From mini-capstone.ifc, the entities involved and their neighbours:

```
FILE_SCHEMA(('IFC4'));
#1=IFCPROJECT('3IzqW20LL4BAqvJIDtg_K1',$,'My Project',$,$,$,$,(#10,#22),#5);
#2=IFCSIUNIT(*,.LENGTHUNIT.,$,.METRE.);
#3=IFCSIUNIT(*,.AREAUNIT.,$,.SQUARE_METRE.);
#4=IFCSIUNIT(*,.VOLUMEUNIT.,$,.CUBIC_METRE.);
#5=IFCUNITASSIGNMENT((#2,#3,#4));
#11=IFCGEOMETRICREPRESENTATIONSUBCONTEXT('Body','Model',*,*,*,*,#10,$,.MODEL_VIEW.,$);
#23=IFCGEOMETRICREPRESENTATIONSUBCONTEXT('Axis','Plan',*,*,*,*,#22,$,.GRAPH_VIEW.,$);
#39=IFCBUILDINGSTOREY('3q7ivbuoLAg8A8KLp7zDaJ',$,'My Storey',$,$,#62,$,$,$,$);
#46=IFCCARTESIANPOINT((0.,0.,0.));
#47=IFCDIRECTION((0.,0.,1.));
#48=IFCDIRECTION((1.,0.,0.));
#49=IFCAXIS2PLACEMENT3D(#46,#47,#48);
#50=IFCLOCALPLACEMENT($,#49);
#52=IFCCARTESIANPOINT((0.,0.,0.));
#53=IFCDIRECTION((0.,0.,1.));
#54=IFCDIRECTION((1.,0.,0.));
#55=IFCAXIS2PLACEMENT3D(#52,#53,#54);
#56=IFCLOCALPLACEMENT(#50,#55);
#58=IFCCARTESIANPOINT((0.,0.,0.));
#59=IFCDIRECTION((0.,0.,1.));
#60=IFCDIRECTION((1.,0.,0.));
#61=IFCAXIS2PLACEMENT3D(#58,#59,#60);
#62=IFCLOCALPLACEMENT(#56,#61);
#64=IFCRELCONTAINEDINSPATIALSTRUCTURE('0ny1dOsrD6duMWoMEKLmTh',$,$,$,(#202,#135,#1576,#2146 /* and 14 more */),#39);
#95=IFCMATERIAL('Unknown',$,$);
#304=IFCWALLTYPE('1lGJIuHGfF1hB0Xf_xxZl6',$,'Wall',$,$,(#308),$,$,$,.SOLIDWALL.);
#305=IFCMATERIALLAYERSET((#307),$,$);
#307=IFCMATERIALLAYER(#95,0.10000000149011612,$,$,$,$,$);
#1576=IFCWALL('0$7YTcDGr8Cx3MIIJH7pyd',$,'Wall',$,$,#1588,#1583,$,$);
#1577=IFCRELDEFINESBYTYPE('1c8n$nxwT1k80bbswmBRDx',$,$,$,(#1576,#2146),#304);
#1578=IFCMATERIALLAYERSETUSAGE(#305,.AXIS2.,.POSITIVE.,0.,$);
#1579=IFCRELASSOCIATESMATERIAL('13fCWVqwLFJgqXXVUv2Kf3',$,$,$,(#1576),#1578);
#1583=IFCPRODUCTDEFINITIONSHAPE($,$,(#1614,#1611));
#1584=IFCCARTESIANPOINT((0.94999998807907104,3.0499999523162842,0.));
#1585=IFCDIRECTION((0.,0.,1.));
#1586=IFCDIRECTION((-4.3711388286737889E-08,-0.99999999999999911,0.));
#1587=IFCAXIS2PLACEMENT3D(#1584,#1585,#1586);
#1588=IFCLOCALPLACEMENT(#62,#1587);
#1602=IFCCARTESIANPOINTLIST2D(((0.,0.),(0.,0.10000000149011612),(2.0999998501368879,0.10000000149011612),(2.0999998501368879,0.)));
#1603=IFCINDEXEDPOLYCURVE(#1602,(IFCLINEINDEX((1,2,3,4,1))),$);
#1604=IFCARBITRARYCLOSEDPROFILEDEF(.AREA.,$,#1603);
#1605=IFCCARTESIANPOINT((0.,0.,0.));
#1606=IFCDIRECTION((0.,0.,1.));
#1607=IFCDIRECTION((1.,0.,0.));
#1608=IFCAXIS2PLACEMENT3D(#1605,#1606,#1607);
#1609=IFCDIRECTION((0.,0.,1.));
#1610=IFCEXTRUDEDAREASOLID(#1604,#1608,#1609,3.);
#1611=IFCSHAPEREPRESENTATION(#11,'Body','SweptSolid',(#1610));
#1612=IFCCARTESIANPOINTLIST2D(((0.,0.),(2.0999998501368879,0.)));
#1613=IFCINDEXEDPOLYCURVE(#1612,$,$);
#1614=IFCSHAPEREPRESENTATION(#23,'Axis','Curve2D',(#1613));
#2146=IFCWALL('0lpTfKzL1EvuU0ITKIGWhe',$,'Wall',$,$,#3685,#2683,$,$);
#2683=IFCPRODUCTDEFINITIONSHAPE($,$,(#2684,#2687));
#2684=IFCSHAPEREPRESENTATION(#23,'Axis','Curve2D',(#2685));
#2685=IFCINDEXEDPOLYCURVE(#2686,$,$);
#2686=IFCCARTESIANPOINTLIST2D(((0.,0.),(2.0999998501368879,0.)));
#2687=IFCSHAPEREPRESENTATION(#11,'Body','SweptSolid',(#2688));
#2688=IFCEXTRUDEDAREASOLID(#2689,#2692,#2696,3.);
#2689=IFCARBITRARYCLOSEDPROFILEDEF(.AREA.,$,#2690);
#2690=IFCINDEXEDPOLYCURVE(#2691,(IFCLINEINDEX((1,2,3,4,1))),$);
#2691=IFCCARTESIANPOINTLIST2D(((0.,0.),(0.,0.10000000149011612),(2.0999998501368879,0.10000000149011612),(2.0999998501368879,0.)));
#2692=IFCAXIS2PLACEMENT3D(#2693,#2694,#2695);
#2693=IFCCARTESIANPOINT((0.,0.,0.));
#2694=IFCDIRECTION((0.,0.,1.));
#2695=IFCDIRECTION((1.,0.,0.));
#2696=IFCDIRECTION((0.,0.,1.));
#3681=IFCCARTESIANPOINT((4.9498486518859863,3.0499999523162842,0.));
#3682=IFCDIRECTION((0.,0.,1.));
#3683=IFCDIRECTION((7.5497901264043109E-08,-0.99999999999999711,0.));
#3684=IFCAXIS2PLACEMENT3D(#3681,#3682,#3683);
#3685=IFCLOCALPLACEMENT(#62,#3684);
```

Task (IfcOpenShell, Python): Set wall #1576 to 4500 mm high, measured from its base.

```python
import ifcopenshell
import ifcopenshell.geom
import ifcopenshell.util.representation
import ifcopenshell.util.shape
import ifcopenshell.util.unit

model = ifcopenshell.open("mini-capstone.ifc")
unit_scale = ifcopenshell.util.unit.calculate_unit_scale(model)
settings = ifcopenshell.geom.settings()


def volume(element):
    """Net volume in cubic metres, openings subtracted."""
    shape = ifcopenshell.geom.create_shape(settings, element)
    return ifcopenshell.util.shape.get_volume(shape.geometry)


wall = model.by_guid("0$7YTcDGr8Cx3MIIJH7pyd")
before = volume(wall)

body = ifcopenshell.util.representation.get_representation(wall, "Model", "Body")
solid = body.Items[0]
old_height = solid.Depth
solid.Depth = 4.5 / unit_scale
after = volume(wall)

print(f"height {old_height:g} -> {solid.Depth:g}, volume {before:.3f} -> {after:.3f} m3")

model.write("mini-capstone_v2.ifc")
```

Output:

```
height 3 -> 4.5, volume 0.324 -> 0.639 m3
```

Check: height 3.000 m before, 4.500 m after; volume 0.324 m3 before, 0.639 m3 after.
